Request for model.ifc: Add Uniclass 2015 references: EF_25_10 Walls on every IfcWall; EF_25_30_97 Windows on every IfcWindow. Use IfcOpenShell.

First a look at what the model holds.

```python
import ifcopenshell

model = ifcopenshell.open("model.ifc")
print(model.schema)
print("classifications:", [c.Name for c in model.by_type("IfcClassification")])
for ifc_class in ("IfcDoor", "IfcRoof", "IfcStair", "IfcWall", "IfcWindow"):
    print(ifc_class, len(model.by_type(ifc_class)))
```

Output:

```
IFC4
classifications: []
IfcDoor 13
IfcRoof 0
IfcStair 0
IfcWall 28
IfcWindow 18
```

```python
import ifcopenshell
import ifcopenshell.api.classification

model = ifcopenshell.open("model.ifc")

system = ifcopenshell.api.classification.add_classification(model, classification="Uniclass 2015")

codes = {
    "IfcWall": ("EF_25_10", "Walls"),
    "IfcWindow": ("EF_25_30_97", "Windows"),
}
for ifc_class, (code, name) in codes.items():
    products = model.by_type(ifc_class)
    ifcopenshell.api.classification.add_reference(
        model, products=products, classification=system, identification=code, name=name
    )
    print(code, len(products))

model.write("model_updated.ifc")
```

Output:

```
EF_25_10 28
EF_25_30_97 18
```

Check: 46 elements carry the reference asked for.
